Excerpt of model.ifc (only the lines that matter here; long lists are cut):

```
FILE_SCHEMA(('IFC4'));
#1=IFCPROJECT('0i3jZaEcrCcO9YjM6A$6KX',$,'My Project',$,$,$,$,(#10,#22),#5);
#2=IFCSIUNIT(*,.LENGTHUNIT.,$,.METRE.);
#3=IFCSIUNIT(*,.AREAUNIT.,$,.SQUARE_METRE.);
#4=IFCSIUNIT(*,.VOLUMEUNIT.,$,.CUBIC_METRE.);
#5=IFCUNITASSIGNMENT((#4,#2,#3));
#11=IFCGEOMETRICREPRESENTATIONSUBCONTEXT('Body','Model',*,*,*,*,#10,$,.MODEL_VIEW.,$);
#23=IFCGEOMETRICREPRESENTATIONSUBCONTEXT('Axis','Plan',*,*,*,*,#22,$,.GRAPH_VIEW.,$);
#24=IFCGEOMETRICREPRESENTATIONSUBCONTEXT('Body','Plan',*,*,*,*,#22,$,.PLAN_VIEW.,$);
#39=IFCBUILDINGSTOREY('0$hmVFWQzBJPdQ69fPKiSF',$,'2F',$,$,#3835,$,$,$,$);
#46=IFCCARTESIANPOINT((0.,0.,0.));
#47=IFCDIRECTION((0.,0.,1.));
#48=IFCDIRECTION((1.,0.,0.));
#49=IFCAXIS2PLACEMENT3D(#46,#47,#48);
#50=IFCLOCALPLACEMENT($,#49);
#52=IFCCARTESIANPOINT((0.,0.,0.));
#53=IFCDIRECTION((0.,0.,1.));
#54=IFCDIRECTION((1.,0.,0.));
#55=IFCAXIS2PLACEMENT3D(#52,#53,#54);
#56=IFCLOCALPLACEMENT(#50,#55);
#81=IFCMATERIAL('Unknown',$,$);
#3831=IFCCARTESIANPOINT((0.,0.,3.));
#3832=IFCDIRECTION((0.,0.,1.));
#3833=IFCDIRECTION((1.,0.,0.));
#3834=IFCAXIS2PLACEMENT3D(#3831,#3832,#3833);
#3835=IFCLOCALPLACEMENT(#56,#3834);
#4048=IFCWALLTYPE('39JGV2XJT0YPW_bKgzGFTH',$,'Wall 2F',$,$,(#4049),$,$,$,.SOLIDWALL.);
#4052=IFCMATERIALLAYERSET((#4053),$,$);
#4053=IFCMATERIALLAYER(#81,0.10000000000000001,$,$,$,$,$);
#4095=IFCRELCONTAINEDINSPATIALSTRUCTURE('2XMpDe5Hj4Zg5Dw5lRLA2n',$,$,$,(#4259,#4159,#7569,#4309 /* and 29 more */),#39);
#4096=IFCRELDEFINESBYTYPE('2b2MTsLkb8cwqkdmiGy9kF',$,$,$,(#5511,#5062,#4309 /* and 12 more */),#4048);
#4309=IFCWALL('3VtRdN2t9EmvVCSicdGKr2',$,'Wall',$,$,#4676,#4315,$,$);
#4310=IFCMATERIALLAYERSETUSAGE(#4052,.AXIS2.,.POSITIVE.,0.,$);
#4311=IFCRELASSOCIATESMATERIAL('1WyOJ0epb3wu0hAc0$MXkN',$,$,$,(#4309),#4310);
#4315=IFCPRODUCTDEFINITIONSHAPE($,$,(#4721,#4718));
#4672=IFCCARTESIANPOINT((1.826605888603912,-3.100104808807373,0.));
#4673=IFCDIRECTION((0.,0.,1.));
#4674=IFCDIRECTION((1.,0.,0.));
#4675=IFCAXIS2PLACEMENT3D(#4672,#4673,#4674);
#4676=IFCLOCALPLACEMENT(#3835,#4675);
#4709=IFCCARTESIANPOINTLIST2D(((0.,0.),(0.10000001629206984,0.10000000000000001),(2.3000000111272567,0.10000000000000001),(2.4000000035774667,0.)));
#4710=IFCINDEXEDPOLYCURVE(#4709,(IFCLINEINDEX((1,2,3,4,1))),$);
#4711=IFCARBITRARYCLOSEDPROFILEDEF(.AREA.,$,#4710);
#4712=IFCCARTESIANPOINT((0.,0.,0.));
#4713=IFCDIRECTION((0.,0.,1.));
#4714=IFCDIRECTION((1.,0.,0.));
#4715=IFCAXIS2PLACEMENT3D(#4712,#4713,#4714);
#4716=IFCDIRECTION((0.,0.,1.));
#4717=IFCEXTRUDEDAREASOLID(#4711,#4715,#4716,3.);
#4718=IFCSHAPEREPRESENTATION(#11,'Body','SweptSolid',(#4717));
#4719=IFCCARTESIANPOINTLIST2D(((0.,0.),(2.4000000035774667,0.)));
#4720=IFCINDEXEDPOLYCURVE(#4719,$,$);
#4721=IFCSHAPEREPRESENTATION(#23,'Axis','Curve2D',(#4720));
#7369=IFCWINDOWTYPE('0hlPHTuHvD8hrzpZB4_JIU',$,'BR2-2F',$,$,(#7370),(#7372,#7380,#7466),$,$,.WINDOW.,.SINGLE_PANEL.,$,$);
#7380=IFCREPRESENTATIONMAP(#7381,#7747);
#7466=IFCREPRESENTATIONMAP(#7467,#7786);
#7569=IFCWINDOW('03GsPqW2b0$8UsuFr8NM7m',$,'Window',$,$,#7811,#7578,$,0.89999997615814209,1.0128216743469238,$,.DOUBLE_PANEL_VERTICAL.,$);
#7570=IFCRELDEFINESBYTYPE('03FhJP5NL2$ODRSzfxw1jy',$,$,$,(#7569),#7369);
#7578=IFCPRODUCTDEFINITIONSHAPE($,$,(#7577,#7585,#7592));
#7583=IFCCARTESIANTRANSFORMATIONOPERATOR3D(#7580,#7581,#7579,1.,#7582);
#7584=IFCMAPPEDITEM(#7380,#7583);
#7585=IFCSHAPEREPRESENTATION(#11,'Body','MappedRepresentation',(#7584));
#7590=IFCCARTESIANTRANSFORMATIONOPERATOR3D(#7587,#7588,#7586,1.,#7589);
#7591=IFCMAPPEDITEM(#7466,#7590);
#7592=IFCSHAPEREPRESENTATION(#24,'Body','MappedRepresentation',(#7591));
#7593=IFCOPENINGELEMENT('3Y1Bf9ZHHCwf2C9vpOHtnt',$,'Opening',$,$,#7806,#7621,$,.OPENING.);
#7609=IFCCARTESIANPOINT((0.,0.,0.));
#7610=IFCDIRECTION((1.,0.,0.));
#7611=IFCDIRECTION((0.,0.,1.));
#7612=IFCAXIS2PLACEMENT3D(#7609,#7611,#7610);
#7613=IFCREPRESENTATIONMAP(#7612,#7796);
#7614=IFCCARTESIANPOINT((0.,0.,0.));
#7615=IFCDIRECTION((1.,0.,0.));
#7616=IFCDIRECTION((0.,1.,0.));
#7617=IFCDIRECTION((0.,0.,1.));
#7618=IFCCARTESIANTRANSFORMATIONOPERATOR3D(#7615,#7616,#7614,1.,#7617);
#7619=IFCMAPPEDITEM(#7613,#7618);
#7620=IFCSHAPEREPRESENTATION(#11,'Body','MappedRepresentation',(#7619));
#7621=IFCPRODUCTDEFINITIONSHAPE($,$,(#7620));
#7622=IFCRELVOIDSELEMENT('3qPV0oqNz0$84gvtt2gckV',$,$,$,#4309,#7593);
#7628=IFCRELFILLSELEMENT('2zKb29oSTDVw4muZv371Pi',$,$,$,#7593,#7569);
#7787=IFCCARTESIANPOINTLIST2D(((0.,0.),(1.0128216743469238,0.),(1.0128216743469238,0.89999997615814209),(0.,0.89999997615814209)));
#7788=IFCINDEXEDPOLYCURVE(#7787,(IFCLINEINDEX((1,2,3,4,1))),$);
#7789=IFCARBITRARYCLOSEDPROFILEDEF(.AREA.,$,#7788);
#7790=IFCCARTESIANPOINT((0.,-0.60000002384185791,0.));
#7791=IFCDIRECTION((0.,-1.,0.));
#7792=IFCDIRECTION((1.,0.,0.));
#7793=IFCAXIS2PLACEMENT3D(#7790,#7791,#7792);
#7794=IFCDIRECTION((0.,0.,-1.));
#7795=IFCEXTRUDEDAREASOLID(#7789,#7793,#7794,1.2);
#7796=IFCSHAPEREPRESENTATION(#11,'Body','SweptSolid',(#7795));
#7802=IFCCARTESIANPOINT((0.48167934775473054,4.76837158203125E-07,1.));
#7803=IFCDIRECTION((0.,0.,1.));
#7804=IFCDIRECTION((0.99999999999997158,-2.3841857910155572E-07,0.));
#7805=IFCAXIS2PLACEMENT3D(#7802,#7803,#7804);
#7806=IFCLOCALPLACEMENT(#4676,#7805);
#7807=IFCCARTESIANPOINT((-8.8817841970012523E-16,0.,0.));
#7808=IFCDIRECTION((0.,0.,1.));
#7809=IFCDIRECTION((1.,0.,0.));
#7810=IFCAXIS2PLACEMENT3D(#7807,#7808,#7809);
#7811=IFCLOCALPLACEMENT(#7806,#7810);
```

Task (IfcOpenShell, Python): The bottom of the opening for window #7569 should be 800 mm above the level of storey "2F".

```python
import numpy as np
import ifcopenshell
import ifcopenshell.api.geometry
import ifcopenshell.geom
import ifcopenshell.util.element
import ifcopenshell.util.placement
import ifcopenshell.util.shape
import ifcopenshell.util.unit

model = ifcopenshell.open("model.ifc")
unit_scale = ifcopenshell.util.unit.calculate_unit_scale(model)

window = model.by_id(7569)
opening = window.FillsVoids[0].RelatingOpeningElement
storey = ifcopenshell.util.element.get_container(window, ifc_class="IfcBuildingStorey")
level = ifcopenshell.util.placement.get_local_placement(storey.ObjectPlacement)[2, 3]

# The opening's origin need not be at the sill, so measure its lowest point.
shape = ifcopenshell.geom.create_shape(ifcopenshell.geom.settings(), opening)
bottom = ifcopenshell.util.shape.get_shape_bottom_elevation(shape, shape.geometry) / unit_scale
dz = level + 0.8 - bottom

shift = np.array([0.0, 0.0, dz])
# The window is placed relative to its opening, so it follows when the opening moves.
matrix = ifcopenshell.util.placement.get_local_placement(opening.ObjectPlacement)
matrix[:3, 3] += shift
ifcopenshell.api.geometry.edit_object_placement(
    model, product=opening, matrix=matrix, is_si=False, should_transform_children=True
)

print(f"moved by {dz * unit_scale:+.3f} m")

model.write("model_v2.ifc")
```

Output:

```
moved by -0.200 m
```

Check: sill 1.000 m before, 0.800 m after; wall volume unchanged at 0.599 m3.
